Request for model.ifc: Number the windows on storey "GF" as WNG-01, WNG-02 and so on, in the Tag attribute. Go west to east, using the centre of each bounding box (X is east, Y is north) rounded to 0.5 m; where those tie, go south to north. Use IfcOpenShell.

First a look at what the model holds.

```python
import ifcopenshell
import ifcopenshell.util.element
import ifcopenshell.util.placement

model = ifcopenshell.open("model.ifc")
print(model.schema)
storey = next(s for s in model.by_type("IfcBuildingStorey") if s.Name == "GF")
windows = [e for e in ifcopenshell.util.element.get_decomposition(storey) if e.is_a("IfcWindow")]
for e in sorted(windows, key=lambda e: e.id()):
    origin = ifcopenshell.util.placement.get_local_placement(e.ObjectPlacement)[:3, 3]
    print(e.id(), e.Tag, e.Name, origin.round(2) + 0.0, sep=" | ")
```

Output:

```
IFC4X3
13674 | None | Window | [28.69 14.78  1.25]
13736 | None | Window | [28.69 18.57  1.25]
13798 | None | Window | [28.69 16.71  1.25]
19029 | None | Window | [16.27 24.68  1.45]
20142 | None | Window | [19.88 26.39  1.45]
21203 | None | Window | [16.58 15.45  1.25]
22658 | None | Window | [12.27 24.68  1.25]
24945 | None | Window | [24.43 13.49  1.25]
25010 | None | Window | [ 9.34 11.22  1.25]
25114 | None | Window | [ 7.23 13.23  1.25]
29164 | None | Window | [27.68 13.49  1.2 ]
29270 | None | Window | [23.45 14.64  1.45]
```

```python
import ifcopenshell
import ifcopenshell.geom
import ifcopenshell.util.element
import ifcopenshell.util.shape

model = ifcopenshell.open("model.ifc")
settings = ifcopenshell.geom.settings()
settings.set("use-world-coords", True)


def centre(element):
    shape = ifcopenshell.geom.create_shape(settings, element)
    return ifcopenshell.util.shape.get_bbox_centroid(shape.geometry)


storey = next(s for s in model.by_type("IfcBuildingStorey") if s.Name == "GF")
windows = [e for e in ifcopenshell.util.element.get_decomposition(storey) if e.is_a("IfcWindow")]

# Insertion points can sit at a corner or the storey origin, so sort by the geometry (in metres).
centres = {e: centre(e) for e in windows}
windows.sort(key=lambda e: (round(centres[e][0] / 0.5), centres[e][1]))

for i, e in enumerate(windows, start=1):
    number = f"WNG-{i:02d}"
    e.Tag = number
    print(e.id(), number)

model.write("model_rev.ifc")
```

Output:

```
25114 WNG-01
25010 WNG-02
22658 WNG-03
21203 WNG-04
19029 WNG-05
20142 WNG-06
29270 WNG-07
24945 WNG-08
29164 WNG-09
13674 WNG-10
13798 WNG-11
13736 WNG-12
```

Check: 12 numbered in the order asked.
